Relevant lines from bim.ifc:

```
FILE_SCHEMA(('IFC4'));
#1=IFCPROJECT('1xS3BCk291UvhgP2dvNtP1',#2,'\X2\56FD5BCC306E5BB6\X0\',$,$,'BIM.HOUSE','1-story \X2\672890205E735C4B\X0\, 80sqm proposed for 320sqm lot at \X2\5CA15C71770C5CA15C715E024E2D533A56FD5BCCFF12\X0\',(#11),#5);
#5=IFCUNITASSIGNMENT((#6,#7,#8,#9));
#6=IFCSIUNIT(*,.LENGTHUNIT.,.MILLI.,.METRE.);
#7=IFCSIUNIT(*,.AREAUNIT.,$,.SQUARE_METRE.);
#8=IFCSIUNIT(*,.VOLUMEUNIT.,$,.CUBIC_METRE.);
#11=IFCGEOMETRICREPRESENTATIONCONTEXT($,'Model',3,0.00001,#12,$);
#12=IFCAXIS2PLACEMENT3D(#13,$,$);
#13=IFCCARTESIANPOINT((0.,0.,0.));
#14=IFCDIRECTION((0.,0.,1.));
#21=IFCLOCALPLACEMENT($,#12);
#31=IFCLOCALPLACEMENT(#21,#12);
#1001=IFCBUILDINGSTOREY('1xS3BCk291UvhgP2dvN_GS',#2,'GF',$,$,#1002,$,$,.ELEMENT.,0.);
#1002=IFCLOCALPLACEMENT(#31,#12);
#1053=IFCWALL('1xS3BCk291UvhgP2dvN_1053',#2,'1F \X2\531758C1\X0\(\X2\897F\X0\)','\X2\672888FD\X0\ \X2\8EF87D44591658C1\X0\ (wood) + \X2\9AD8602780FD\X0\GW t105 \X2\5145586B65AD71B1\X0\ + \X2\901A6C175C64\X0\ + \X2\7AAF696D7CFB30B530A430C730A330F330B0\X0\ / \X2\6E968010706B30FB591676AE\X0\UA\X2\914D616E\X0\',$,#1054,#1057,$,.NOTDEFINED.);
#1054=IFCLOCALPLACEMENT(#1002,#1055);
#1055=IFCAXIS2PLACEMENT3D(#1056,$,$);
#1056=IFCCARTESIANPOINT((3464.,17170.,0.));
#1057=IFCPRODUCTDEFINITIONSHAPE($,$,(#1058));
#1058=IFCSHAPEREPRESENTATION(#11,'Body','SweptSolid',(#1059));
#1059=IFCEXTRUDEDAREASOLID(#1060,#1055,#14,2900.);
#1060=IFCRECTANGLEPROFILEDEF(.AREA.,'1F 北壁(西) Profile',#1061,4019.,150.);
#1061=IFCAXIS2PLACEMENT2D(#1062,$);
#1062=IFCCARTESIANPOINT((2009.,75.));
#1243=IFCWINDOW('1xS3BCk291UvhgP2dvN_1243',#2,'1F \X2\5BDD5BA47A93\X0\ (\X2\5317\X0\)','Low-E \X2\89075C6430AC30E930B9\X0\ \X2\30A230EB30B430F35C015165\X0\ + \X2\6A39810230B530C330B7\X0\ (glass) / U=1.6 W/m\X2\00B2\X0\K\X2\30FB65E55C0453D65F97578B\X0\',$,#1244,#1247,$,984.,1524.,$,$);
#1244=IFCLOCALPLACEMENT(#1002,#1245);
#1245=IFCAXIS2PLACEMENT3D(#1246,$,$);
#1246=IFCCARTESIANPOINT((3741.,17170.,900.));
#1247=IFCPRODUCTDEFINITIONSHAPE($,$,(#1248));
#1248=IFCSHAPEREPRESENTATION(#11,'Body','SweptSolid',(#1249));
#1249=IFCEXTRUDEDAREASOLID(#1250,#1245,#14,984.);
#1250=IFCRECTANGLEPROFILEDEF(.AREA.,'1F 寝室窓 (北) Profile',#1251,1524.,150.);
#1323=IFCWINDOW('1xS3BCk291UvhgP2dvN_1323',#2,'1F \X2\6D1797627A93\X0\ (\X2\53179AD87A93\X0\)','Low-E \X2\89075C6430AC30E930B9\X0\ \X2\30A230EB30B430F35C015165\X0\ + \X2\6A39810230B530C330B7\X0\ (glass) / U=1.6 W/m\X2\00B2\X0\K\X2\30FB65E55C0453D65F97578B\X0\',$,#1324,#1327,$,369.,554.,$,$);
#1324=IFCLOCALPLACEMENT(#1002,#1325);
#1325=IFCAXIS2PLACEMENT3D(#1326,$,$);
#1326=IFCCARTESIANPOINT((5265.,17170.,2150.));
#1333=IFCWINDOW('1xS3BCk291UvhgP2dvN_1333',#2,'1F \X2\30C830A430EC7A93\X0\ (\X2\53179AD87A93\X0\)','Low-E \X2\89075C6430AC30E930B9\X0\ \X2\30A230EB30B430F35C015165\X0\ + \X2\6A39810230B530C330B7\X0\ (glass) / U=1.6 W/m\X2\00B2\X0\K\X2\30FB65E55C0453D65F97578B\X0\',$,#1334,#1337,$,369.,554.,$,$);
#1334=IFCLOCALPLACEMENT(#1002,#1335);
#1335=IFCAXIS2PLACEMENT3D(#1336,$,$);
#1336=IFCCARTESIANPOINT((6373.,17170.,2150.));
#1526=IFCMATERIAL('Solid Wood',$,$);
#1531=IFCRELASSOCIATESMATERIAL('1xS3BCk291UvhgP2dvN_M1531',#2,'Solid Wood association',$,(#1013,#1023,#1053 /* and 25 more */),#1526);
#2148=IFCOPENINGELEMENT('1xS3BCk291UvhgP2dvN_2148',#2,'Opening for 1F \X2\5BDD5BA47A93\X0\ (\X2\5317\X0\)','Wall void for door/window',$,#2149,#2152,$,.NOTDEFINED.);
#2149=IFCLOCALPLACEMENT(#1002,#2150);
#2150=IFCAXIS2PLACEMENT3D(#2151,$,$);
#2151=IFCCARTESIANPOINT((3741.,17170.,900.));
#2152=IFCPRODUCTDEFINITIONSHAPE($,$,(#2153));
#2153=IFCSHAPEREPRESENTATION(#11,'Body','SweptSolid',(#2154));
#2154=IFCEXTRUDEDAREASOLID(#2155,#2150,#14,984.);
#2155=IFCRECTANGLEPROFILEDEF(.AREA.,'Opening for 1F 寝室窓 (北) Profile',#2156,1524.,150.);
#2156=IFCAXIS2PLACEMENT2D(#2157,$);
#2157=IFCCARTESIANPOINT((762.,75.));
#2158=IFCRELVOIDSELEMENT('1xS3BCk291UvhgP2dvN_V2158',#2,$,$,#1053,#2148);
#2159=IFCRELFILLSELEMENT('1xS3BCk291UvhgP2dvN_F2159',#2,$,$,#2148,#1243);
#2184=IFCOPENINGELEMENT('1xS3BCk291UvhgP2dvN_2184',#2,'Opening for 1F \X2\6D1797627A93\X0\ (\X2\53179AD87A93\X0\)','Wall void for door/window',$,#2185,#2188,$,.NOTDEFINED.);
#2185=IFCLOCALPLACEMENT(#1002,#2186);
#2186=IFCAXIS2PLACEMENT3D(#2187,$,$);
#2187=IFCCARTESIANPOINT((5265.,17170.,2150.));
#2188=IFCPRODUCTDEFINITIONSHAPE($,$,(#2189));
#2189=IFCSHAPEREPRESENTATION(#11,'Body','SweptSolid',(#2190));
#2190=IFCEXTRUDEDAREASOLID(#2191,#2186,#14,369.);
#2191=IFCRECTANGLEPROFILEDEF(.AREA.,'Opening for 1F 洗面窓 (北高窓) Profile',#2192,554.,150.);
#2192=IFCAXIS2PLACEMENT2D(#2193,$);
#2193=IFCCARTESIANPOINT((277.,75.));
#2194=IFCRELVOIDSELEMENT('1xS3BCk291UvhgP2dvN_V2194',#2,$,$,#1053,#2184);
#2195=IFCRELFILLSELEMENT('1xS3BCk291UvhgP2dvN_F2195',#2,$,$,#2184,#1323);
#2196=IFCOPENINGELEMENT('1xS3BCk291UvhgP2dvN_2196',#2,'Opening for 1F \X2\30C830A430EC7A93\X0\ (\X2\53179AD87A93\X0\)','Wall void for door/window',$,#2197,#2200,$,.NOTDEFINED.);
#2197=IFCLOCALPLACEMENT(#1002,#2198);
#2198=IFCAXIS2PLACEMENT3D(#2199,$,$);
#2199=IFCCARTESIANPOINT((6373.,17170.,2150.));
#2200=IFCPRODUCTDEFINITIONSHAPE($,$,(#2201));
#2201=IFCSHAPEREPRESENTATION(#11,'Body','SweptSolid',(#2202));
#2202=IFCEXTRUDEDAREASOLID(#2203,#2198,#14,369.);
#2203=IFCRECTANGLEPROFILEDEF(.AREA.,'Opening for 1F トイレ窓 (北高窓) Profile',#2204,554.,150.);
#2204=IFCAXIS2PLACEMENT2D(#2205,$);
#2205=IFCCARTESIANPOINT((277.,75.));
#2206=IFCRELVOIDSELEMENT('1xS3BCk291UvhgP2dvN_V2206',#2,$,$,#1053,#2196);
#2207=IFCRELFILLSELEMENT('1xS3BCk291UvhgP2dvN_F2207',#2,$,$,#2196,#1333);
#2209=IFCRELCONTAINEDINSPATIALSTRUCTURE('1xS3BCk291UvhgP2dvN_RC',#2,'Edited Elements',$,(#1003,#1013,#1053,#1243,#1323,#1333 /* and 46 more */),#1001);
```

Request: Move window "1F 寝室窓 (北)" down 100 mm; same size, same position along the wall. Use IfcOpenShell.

```python
import numpy as np
import ifcopenshell
import ifcopenshell.api.geometry
import ifcopenshell.util.placement
import ifcopenshell.util.unit

model = ifcopenshell.open("bim.ifc")
unit_scale = ifcopenshell.util.unit.calculate_unit_scale(model)

window = model.by_id(1243)
opening = window.FillsVoids[0].RelatingOpeningElement
dz = -0.1 / unit_scale

shift = np.array([0.0, 0.0, dz])
# The window is not placed relative to its opening, so move both.
for product in (opening, window):
    matrix = ifcopenshell.util.placement.get_local_placement(product.ObjectPlacement)
    matrix[:3, 3] += shift
    ifcopenshell.api.geometry.edit_object_placement(model, product=product, matrix=matrix, is_si=False)

print(f"moved by {dz * unit_scale:+.3f} m")

model.write("bim_edited.ifc")
```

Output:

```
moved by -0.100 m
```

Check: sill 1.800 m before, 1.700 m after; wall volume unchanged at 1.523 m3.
